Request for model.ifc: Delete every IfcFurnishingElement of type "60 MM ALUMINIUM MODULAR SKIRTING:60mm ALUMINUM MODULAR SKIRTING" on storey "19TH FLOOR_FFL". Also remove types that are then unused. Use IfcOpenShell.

First a look at what the model holds.

```python
import ifcopenshell
import ifcopenshell.util.element

model = ifcopenshell.open("model.ifc")
print(model.schema)
storey = next(s for s in model.by_type("IfcBuildingStorey") if s.Name == "19TH FLOOR_FFL")
furniture = [e for e in ifcopenshell.util.element.get_decomposition(storey) if e.is_a("IfcFurnishingElement")]
seen = {}
for e in furniture:
    element_type = ifcopenshell.util.element.get_type(e)
    name = element_type.Name if element_type not in (None, e) else None
    seen[name] = seen.get(name, 0) + 1
for name, count in sorted(seen.items(), key=str):
    print(count, "x", name)
```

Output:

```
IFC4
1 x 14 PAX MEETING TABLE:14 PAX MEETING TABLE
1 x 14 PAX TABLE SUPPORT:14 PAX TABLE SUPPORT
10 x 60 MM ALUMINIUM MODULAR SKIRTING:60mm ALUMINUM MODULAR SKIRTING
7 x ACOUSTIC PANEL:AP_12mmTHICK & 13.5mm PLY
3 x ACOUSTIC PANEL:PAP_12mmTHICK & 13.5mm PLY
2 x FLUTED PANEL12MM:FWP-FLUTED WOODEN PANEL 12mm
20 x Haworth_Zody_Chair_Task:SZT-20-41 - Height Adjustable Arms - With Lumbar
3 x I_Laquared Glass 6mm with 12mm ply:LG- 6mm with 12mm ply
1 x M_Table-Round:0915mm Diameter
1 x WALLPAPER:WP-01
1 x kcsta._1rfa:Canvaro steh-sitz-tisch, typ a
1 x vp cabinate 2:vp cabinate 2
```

```python
import ifcopenshell
import ifcopenshell.api.root
import ifcopenshell.util.element

model = ifcopenshell.open("model.ifc")

storey = next(s for s in model.by_type("IfcBuildingStorey") if s.Name == "19TH FLOOR_FFL")
furniture = [e for e in ifcopenshell.util.element.get_decomposition(storey) if e.is_a("IfcFurnishingElement")]
targets = [e for e in furniture if (t := ifcopenshell.util.element.get_type(e)) not in (None, e) and t.Name == "60 MM ALUMINIUM MODULAR SKIRTING:60mm ALUMINUM MODULAR SKIRTING"]
types = {ifcopenshell.util.element.get_type(e) for e in targets} - {None, *targets}

for e in targets:
    ifcopenshell.api.root.remove_product(model, product=e)
print(len(targets), "removed")

unused = [t for t in types if not ifcopenshell.util.element.get_types(t)]
for t in unused:
    ifcopenshell.api.root.remove_product(model, product=t)
print(len(unused), "unused types removed")

model.write("model_rev.ifc")
```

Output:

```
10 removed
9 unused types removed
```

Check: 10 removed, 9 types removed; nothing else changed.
